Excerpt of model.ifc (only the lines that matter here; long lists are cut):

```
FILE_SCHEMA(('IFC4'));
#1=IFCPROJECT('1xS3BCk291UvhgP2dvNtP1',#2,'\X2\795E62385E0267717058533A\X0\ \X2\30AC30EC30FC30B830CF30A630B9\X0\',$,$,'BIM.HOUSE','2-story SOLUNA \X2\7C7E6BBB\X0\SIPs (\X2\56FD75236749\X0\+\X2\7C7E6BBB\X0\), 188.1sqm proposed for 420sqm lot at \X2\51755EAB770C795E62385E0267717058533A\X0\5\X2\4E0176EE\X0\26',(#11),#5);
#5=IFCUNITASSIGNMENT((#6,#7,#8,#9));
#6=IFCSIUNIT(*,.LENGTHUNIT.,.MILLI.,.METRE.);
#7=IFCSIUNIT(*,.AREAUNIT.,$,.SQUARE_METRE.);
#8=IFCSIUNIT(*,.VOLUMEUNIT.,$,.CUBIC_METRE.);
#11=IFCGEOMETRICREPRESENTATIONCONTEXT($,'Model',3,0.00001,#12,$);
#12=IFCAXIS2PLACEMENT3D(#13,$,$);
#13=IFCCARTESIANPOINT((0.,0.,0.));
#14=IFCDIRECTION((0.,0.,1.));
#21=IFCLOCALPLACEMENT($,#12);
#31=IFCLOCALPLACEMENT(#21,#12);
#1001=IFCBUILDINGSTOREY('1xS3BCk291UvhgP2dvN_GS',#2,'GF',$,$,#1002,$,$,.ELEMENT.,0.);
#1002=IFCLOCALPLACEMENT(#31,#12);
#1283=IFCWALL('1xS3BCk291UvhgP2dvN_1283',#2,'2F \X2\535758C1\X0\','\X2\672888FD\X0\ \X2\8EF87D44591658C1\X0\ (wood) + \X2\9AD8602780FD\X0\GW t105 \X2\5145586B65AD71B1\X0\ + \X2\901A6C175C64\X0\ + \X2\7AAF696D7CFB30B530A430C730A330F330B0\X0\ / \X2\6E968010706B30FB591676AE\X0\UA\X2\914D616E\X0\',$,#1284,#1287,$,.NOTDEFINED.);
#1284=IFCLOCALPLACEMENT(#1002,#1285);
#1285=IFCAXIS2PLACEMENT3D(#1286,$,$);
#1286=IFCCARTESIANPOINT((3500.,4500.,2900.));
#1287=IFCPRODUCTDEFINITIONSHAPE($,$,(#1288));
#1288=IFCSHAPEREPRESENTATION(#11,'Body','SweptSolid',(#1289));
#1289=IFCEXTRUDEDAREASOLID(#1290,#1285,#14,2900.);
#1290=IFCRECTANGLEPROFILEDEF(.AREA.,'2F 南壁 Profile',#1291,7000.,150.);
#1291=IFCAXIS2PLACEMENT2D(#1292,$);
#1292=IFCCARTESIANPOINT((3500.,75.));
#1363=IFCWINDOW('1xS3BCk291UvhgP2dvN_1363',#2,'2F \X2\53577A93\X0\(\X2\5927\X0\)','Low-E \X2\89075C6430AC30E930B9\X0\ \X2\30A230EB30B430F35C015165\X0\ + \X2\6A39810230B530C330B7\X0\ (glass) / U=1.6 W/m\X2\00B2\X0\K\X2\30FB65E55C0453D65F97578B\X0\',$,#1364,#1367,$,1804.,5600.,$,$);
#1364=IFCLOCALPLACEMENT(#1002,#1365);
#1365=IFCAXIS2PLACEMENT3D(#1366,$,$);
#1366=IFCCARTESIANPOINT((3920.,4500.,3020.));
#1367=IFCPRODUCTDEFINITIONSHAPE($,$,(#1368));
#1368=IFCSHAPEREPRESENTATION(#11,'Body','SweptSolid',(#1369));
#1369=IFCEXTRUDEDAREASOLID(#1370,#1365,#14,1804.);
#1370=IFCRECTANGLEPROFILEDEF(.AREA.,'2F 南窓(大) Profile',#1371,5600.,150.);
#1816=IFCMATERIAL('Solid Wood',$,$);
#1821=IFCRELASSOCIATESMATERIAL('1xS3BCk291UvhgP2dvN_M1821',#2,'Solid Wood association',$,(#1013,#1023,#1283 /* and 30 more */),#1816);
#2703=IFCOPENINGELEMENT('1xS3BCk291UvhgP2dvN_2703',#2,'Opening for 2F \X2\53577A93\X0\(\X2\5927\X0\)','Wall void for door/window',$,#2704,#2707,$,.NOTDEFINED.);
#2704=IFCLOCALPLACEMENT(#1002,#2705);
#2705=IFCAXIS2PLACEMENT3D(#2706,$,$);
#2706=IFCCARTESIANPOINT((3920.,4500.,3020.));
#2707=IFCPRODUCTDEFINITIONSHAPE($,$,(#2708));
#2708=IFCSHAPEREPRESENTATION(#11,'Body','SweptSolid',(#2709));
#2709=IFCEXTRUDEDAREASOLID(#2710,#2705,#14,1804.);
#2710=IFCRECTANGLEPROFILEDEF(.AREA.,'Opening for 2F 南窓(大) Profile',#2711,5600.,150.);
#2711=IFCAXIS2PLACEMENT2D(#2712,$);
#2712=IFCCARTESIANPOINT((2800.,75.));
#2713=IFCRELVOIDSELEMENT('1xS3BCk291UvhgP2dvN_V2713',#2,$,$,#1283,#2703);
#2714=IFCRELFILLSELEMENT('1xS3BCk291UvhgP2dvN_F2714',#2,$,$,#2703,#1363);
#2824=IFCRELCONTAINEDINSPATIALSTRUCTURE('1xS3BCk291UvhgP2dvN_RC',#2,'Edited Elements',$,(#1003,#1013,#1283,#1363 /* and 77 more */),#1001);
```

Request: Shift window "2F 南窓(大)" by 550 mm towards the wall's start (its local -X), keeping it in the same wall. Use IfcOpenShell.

```python
import ifcopenshell
import ifcopenshell.api.geometry
import ifcopenshell.util.placement
import ifcopenshell.util.unit

model = ifcopenshell.open("model.ifc")
unit_scale = ifcopenshell.util.unit.calculate_unit_scale(model)

window = model.by_guid("1xS3BCk291UvhgP2dvN_1363")
opening = window.FillsVoids[0].RelatingOpeningElement
wall = opening.VoidsElements[0].RelatingBuildingElement

wall_matrix = ifcopenshell.util.placement.get_local_placement(wall.ObjectPlacement)
shift = wall_matrix[:3, 0] * -0.55 / unit_scale
before = ifcopenshell.util.placement.get_local_placement(window.ObjectPlacement)[:3, 3].copy()

# The window is not placed relative to its opening, so move both.
for product in (opening, window):
    matrix = ifcopenshell.util.placement.get_local_placement(product.ObjectPlacement)
    matrix[:3, 3] += shift
    ifcopenshell.api.geometry.edit_object_placement(model, product=product, matrix=matrix, is_si=False)

after = ifcopenshell.util.placement.get_local_placement(window.ObjectPlacement)[:3, 3]
print("window moved by", (after - before).round(3) + 0.0)

model.write("model_rev.ifc")
```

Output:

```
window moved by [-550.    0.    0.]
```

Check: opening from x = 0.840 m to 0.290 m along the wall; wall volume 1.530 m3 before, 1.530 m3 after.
